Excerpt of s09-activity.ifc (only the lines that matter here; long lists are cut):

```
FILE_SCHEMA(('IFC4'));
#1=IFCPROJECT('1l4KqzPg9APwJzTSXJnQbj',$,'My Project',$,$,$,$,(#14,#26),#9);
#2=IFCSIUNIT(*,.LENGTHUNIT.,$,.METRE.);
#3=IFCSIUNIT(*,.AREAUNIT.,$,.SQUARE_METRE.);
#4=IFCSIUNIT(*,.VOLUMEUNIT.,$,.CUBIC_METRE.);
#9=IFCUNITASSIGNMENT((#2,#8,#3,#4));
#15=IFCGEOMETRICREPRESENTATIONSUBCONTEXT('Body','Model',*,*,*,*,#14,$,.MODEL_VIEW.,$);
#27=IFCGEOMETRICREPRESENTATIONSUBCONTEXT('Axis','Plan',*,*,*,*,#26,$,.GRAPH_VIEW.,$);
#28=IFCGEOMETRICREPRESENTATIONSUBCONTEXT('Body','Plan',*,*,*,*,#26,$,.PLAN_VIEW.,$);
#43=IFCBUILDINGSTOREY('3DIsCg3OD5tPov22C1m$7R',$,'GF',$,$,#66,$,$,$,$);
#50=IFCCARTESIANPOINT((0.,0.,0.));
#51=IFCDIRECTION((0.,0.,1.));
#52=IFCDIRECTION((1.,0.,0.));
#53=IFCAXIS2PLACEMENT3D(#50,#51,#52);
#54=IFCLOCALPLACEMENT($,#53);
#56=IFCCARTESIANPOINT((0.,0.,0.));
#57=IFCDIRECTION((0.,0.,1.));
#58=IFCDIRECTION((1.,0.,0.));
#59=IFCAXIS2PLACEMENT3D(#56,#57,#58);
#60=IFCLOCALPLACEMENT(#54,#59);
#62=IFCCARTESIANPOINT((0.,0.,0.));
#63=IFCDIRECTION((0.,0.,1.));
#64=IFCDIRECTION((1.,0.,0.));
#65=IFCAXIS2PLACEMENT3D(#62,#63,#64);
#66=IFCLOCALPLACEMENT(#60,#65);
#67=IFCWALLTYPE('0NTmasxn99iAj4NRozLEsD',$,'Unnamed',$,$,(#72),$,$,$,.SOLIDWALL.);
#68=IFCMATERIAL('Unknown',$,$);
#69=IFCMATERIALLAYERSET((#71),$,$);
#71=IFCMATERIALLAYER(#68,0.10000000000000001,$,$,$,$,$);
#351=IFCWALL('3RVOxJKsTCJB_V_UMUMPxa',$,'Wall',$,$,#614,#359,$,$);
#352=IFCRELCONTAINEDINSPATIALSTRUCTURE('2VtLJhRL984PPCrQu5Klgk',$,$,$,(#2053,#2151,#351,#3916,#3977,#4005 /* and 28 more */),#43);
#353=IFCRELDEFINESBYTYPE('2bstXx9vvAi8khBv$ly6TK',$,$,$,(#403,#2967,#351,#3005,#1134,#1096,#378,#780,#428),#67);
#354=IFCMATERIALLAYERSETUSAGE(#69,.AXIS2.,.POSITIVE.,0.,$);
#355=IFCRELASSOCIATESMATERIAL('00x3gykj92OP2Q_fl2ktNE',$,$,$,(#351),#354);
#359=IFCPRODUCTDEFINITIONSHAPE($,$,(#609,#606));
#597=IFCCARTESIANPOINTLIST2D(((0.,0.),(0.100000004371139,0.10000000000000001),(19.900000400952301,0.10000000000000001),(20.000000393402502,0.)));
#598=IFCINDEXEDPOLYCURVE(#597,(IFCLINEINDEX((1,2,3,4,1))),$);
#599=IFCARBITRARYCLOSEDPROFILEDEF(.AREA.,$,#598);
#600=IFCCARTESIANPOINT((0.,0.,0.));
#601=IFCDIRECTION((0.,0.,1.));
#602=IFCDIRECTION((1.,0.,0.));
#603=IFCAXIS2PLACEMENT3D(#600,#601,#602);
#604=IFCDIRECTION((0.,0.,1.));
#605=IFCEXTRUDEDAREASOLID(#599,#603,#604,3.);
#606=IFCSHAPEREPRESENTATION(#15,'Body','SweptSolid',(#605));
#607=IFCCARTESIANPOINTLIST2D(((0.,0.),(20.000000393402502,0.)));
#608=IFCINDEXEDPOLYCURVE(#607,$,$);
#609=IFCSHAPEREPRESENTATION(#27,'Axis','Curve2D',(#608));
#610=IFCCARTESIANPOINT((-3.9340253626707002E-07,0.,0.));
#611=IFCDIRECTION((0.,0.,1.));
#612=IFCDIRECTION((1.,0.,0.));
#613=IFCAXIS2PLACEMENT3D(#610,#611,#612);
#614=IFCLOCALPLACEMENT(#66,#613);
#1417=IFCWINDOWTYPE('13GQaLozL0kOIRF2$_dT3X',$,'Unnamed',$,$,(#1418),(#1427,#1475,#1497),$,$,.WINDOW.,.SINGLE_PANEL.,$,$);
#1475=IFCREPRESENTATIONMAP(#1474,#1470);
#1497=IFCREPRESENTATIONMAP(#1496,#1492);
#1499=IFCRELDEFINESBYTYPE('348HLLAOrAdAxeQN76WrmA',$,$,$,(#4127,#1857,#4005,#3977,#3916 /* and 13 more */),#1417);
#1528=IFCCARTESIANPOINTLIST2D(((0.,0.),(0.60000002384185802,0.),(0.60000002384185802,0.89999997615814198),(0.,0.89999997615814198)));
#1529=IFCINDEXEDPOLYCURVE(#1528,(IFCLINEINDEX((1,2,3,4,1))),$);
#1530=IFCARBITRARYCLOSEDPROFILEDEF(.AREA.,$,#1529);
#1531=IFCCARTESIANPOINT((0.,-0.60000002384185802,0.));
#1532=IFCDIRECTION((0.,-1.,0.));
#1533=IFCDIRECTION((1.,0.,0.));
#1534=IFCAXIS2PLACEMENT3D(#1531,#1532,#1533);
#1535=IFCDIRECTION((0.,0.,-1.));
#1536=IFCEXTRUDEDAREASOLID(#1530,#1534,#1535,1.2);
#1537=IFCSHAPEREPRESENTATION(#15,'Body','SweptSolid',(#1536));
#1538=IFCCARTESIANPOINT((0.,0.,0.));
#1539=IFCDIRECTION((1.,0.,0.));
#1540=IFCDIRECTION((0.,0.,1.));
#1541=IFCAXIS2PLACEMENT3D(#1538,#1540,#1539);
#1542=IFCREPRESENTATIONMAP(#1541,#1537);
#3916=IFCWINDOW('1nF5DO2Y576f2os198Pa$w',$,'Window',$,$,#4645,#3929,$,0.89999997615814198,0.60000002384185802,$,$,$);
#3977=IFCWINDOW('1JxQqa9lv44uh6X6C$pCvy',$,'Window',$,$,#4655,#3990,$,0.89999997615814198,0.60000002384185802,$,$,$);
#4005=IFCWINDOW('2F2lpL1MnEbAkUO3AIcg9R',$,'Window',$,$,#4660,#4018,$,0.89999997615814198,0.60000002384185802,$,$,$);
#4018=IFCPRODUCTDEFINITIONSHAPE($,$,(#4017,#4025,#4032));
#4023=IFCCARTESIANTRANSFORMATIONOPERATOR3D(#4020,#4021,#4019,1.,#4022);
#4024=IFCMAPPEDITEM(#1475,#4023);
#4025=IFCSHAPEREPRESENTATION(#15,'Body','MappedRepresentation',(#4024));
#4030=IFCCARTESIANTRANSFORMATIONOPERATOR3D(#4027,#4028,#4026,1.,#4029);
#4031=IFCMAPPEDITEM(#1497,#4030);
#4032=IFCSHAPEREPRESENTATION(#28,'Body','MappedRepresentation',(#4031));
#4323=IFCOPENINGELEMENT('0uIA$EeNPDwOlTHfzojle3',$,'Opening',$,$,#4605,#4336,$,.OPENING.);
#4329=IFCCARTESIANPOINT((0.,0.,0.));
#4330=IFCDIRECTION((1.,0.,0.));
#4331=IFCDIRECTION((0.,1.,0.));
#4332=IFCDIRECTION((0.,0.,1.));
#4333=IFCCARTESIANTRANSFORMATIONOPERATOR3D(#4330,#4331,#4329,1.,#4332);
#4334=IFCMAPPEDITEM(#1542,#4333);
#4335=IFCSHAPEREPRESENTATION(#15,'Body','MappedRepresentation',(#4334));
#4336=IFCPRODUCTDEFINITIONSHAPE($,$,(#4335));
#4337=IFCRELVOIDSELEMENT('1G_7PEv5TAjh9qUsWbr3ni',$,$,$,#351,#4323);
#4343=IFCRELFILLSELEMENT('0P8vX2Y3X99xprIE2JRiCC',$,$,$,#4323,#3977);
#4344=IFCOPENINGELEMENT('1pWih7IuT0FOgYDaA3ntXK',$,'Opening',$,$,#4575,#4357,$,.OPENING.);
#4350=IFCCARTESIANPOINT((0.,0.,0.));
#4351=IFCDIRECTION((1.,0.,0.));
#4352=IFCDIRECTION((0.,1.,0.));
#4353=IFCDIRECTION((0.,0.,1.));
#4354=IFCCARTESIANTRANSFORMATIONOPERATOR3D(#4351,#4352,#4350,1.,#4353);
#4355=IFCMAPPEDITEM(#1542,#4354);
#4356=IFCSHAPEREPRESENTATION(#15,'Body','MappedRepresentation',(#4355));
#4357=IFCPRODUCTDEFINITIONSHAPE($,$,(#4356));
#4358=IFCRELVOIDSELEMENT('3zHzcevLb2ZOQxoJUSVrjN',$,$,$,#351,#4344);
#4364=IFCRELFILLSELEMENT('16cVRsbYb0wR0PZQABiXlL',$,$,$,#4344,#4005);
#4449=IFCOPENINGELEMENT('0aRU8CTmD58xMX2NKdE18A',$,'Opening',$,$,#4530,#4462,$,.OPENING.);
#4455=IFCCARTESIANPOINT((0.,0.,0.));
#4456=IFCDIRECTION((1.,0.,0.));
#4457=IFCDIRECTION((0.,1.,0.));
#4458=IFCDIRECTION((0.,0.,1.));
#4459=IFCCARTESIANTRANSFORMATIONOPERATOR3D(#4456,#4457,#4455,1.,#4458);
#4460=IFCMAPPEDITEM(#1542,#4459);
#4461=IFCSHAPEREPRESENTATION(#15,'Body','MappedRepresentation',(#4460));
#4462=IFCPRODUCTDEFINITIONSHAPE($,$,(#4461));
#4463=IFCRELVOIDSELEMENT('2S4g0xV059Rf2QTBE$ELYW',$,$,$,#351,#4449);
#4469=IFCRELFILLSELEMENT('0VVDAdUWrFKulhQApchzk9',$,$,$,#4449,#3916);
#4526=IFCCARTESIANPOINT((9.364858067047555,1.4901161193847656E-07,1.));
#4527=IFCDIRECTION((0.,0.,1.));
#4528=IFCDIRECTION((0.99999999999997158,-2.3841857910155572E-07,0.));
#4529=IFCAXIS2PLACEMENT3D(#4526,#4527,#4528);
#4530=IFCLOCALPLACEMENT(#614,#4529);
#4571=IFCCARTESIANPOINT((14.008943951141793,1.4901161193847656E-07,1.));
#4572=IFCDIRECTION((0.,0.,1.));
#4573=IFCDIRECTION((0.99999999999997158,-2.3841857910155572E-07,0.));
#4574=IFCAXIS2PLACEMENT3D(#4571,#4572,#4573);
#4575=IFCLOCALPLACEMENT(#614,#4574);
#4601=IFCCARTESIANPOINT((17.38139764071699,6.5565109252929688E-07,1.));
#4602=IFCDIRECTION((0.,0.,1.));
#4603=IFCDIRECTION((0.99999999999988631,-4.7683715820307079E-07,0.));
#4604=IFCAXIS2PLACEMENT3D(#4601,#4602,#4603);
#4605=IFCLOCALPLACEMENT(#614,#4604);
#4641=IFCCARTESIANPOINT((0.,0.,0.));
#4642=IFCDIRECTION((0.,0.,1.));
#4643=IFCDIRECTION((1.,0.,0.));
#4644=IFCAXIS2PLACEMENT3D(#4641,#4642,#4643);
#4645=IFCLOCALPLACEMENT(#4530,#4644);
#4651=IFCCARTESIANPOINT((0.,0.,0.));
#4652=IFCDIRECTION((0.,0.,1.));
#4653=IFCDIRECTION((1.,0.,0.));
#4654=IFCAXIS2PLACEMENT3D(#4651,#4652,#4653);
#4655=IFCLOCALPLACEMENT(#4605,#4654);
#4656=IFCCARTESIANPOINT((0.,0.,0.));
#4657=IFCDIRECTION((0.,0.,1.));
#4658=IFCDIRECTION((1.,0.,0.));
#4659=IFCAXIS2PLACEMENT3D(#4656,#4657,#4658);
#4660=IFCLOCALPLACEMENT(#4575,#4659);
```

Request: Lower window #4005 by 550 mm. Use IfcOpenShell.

```python
import numpy as np
import ifcopenshell
import ifcopenshell.api.geometry
import ifcopenshell.util.placement
import ifcopenshell.util.unit

model = ifcopenshell.open("s09-activity.ifc")
unit_scale = ifcopenshell.util.unit.calculate_unit_scale(model)

window = model.by_guid("2F2lpL1MnEbAkUO3AIcg9R")
opening = window.FillsVoids[0].RelatingOpeningElement
dz = -0.55

shift = np.array([0.0, 0.0, dz])
# The window is placed relative to its opening, so it follows when the opening moves.
matrix = ifcopenshell.util.placement.get_local_placement(opening.ObjectPlacement)
matrix[:3, 3] += shift
ifcopenshell.api.geometry.edit_object_placement(
    model, product=opening, matrix=matrix, is_si=False, should_transform_children=True
)

print(f"moved by {dz * unit_scale:+.3f} m")

model.write("s09-activity-out.ifc")
```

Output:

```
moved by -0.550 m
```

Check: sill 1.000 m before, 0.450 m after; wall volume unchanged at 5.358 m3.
